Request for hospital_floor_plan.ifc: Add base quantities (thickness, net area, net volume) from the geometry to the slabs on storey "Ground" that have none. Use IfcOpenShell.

First a look at what the model holds.

```python
import ifcopenshell
import ifcopenshell.util.element
import ifcopenshell.util.unit

model = ifcopenshell.open("hospital_floor_plan.ifc")
print(model.schema)
for unit_type in ("LENGTHUNIT", "AREAUNIT", "VOLUMEUNIT"):
    print(unit_type, ifcopenshell.util.unit.calculate_unit_scale(model, unit_type))
storey = next(s for s in model.by_type("IfcBuildingStorey") if s.Name == "Ground")
slabs = [e for e in ifcopenshell.util.element.get_decomposition(storey) if e.is_a("IfcSlab")]
for e in sorted(slabs, key=lambda e: e.id()):
    print(e.id(), e.is_a(), e.Name, list(ifcopenshell.util.element.get_psets(e, qtos_only=True)), sep=" | ")
```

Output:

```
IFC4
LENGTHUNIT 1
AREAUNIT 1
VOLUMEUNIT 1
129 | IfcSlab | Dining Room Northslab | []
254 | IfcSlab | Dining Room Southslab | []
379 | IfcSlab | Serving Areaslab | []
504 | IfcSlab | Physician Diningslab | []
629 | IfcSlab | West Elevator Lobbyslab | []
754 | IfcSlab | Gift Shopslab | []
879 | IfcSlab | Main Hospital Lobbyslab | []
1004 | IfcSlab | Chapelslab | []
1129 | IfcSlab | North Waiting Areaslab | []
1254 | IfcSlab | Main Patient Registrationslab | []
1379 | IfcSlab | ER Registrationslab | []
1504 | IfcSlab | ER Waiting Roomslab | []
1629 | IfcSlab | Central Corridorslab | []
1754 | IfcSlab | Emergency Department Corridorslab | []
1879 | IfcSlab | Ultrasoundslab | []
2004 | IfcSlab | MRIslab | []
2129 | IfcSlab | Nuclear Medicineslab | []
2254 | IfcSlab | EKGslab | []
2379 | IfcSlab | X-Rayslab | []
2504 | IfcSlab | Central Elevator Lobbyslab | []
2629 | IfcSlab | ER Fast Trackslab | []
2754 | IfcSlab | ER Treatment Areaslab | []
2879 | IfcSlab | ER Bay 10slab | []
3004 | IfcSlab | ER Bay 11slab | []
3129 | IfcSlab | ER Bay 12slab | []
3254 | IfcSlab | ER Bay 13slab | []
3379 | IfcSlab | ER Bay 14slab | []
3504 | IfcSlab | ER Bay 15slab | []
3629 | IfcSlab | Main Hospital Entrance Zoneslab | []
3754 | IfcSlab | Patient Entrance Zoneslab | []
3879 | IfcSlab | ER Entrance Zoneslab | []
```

```python
import ifcopenshell
import ifcopenshell.api.pset
import ifcopenshell.geom
import ifcopenshell.util.element
import ifcopenshell.util.shape
import ifcopenshell.util.unit

model = ifcopenshell.open("hospital_floor_plan.ifc")
unit_scale = ifcopenshell.util.unit.calculate_unit_scale(model)
area_scale = ifcopenshell.util.unit.calculate_unit_scale(model, "AREAUNIT")
volume_scale = ifcopenshell.util.unit.calculate_unit_scale(model, "VOLUMEUNIT")
settings = ifcopenshell.geom.settings()

storey = next(s for s in model.by_type("IfcBuildingStorey") if s.Name == "Ground")
slabs = [e for e in ifcopenshell.util.element.get_decomposition(storey) if e.is_a("IfcSlab")]

for e in sorted(slabs, key=lambda e: e.id()):
    if ifcopenshell.util.element.get_psets(e, qtos_only=True, should_inherit=False):
        continue
    # Geometry comes back in metres, in the element's own axes.
    shape = ifcopenshell.geom.create_shape(settings, e)
    values = {
        "Width": ifcopenshell.util.shape.get_z(shape.geometry) / unit_scale,
        "NetArea": ifcopenshell.util.shape.get_footprint_area(shape.geometry) / area_scale,
        "NetVolume": ifcopenshell.util.shape.get_volume(shape.geometry) / volume_scale,
    }
    qto = ifcopenshell.api.pset.add_qto(model, product=e, name="Qto_SlabBaseQuantities")
    ifcopenshell.api.pset.edit_qto(model, qto=qto, properties=values)
    print(e.id(), {k: round(v, 3) for k, v in values.items()})

model.write("hospital_floor_plan_edited.ifc")
```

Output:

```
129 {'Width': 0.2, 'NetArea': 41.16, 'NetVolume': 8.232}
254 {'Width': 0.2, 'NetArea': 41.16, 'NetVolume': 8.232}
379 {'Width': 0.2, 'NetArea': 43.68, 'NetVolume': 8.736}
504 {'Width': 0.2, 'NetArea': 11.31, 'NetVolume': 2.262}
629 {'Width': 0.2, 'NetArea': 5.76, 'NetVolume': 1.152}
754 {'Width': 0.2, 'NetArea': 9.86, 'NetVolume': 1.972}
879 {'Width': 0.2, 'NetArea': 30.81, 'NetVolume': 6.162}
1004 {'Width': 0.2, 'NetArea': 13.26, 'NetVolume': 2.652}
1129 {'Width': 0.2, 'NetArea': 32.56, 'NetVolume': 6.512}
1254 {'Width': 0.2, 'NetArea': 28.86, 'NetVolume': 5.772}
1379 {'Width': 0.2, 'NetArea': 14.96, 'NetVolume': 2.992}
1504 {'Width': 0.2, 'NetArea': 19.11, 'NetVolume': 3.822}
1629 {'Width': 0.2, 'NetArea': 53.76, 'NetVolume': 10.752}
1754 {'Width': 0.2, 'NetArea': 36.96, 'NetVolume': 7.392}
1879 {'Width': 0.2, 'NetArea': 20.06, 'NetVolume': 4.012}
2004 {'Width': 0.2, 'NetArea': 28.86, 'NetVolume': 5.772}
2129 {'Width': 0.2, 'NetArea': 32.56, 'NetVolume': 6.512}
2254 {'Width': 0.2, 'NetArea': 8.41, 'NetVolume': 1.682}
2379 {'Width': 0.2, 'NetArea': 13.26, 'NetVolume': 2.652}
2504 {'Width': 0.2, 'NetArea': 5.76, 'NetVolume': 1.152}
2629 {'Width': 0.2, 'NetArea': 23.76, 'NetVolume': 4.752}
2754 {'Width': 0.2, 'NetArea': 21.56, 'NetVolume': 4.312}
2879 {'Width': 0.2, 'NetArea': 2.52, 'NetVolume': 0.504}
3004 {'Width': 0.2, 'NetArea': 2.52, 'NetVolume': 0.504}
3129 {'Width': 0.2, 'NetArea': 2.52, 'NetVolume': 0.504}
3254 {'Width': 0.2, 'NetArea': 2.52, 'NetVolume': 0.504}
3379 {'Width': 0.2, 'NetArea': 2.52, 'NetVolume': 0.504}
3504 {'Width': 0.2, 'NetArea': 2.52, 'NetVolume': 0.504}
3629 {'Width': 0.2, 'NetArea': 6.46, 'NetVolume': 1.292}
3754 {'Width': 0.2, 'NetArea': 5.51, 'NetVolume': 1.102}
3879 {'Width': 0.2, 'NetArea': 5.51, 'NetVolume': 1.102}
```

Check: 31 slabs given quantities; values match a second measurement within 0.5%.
